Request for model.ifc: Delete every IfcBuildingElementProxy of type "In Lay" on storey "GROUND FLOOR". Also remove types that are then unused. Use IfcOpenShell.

First a look at what the model holds.

```python
import ifcopenshell
import ifcopenshell.util.element

model = ifcopenshell.open("model.ifc")
print(model.schema)
storey = next(s for s in model.by_type("IfcBuildingStorey") if s.Name == "GROUND FLOOR")
proxies = [e for e in ifcopenshell.util.element.get_decomposition(storey) if e.is_a("IfcBuildingElementProxy")]
seen = {}
for e in proxies:
    element_type = ifcopenshell.util.element.get_type(e)
    name = element_type.Name if element_type not in (None, e) else None
    seen[name] = seen.get(name, 0) + 1
for name, count in sorted(seen.items(), key=str):
    print(count, "x", name)
```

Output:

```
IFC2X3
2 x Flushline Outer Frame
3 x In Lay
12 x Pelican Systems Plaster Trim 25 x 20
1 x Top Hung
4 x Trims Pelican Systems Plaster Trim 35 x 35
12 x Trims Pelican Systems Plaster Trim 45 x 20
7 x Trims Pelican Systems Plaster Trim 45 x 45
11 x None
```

```python
import ifcopenshell
import ifcopenshell.api.root
import ifcopenshell.util.element

model = ifcopenshell.open("model.ifc")

storey = next(s for s in model.by_type("IfcBuildingStorey") if s.Name == "GROUND FLOOR")
proxies = [e for e in ifcopenshell.util.element.get_decomposition(storey) if e.is_a("IfcBuildingElementProxy")]
targets = [e for e in proxies if (t := ifcopenshell.util.element.get_type(e)) not in (None, e) and t.Name == "In Lay"]
types = {ifcopenshell.util.element.get_type(e) for e in targets} - {None, *targets}

for e in targets:
    ifcopenshell.api.root.remove_product(model, product=e)
print(len(targets), "removed")

unused = [t for t in types if not ifcopenshell.util.element.get_types(t)]
for t in unused:
    ifcopenshell.api.root.remove_product(model, product=t)
print(len(unused), "unused types removed")

model.write("model_v2.ifc")
```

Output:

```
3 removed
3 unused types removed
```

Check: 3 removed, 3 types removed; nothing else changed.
